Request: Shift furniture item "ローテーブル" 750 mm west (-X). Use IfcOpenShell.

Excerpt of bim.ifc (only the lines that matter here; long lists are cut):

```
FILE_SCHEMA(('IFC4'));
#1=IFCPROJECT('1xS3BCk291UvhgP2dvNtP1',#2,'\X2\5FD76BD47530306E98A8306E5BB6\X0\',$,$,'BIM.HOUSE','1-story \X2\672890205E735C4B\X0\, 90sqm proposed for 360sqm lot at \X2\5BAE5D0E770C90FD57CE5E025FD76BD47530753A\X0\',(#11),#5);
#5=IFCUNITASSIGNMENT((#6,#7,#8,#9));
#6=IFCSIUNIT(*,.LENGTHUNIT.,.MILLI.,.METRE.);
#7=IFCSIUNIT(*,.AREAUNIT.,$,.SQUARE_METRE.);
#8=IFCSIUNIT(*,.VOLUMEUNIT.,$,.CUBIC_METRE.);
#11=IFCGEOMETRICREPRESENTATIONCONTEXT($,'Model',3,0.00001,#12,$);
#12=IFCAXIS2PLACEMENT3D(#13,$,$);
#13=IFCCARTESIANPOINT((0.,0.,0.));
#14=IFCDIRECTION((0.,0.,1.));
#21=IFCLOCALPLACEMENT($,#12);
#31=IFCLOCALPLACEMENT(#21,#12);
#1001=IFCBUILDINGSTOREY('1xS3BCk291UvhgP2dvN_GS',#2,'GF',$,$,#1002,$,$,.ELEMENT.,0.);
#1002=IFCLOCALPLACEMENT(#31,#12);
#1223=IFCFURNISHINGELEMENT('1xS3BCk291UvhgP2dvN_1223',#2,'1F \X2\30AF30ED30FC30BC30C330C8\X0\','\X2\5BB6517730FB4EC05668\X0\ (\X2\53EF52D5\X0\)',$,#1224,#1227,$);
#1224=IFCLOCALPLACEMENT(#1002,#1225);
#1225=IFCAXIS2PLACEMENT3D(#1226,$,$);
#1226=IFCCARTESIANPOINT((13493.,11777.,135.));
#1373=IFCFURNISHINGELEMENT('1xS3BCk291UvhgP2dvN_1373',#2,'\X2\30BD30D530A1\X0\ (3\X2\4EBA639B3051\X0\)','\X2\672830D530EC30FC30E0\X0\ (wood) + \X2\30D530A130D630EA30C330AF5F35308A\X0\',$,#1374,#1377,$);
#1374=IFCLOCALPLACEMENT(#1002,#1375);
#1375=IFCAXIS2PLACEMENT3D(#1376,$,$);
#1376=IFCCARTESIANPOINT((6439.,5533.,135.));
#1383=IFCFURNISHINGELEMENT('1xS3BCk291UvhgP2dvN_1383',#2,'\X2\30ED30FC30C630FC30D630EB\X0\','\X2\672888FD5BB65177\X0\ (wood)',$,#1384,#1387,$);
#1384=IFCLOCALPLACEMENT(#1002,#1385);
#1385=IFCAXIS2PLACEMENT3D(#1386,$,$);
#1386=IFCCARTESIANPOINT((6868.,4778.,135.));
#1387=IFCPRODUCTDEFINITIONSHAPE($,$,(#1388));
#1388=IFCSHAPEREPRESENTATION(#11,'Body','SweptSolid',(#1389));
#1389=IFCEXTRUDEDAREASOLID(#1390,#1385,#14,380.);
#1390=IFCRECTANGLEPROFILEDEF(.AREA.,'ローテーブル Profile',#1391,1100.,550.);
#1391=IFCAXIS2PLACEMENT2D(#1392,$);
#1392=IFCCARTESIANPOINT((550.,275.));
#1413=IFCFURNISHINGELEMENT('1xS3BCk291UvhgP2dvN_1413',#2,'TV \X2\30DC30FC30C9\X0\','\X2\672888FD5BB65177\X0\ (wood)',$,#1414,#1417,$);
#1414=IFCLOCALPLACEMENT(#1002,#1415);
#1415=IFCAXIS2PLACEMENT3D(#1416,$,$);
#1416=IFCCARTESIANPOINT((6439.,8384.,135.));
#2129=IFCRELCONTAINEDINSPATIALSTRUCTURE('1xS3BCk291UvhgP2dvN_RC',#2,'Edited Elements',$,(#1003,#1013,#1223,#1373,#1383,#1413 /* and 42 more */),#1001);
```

```python
import ifcopenshell
import ifcopenshell.api.geometry
import ifcopenshell.util.placement
import ifcopenshell.util.unit

model = ifcopenshell.open("bim.ifc")
unit_scale = ifcopenshell.util.unit.calculate_unit_scale(model)

item = model.by_guid("1xS3BCk291UvhgP2dvN_1383")
matrix = ifcopenshell.util.placement.get_local_placement(item.ObjectPlacement)
matrix[0, 3] -= 0.75 / unit_scale
ifcopenshell.api.geometry.edit_object_placement(model, product=item, matrix=matrix, is_si=False)

print(ifcopenshell.util.placement.get_local_placement(item.ObjectPlacement).round(3) + 0.0)

model.write("bim-out.ifc")
```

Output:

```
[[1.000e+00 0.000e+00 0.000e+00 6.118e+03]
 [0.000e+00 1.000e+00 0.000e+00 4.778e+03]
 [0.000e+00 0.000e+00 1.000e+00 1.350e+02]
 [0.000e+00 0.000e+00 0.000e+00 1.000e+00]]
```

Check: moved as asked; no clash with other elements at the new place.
